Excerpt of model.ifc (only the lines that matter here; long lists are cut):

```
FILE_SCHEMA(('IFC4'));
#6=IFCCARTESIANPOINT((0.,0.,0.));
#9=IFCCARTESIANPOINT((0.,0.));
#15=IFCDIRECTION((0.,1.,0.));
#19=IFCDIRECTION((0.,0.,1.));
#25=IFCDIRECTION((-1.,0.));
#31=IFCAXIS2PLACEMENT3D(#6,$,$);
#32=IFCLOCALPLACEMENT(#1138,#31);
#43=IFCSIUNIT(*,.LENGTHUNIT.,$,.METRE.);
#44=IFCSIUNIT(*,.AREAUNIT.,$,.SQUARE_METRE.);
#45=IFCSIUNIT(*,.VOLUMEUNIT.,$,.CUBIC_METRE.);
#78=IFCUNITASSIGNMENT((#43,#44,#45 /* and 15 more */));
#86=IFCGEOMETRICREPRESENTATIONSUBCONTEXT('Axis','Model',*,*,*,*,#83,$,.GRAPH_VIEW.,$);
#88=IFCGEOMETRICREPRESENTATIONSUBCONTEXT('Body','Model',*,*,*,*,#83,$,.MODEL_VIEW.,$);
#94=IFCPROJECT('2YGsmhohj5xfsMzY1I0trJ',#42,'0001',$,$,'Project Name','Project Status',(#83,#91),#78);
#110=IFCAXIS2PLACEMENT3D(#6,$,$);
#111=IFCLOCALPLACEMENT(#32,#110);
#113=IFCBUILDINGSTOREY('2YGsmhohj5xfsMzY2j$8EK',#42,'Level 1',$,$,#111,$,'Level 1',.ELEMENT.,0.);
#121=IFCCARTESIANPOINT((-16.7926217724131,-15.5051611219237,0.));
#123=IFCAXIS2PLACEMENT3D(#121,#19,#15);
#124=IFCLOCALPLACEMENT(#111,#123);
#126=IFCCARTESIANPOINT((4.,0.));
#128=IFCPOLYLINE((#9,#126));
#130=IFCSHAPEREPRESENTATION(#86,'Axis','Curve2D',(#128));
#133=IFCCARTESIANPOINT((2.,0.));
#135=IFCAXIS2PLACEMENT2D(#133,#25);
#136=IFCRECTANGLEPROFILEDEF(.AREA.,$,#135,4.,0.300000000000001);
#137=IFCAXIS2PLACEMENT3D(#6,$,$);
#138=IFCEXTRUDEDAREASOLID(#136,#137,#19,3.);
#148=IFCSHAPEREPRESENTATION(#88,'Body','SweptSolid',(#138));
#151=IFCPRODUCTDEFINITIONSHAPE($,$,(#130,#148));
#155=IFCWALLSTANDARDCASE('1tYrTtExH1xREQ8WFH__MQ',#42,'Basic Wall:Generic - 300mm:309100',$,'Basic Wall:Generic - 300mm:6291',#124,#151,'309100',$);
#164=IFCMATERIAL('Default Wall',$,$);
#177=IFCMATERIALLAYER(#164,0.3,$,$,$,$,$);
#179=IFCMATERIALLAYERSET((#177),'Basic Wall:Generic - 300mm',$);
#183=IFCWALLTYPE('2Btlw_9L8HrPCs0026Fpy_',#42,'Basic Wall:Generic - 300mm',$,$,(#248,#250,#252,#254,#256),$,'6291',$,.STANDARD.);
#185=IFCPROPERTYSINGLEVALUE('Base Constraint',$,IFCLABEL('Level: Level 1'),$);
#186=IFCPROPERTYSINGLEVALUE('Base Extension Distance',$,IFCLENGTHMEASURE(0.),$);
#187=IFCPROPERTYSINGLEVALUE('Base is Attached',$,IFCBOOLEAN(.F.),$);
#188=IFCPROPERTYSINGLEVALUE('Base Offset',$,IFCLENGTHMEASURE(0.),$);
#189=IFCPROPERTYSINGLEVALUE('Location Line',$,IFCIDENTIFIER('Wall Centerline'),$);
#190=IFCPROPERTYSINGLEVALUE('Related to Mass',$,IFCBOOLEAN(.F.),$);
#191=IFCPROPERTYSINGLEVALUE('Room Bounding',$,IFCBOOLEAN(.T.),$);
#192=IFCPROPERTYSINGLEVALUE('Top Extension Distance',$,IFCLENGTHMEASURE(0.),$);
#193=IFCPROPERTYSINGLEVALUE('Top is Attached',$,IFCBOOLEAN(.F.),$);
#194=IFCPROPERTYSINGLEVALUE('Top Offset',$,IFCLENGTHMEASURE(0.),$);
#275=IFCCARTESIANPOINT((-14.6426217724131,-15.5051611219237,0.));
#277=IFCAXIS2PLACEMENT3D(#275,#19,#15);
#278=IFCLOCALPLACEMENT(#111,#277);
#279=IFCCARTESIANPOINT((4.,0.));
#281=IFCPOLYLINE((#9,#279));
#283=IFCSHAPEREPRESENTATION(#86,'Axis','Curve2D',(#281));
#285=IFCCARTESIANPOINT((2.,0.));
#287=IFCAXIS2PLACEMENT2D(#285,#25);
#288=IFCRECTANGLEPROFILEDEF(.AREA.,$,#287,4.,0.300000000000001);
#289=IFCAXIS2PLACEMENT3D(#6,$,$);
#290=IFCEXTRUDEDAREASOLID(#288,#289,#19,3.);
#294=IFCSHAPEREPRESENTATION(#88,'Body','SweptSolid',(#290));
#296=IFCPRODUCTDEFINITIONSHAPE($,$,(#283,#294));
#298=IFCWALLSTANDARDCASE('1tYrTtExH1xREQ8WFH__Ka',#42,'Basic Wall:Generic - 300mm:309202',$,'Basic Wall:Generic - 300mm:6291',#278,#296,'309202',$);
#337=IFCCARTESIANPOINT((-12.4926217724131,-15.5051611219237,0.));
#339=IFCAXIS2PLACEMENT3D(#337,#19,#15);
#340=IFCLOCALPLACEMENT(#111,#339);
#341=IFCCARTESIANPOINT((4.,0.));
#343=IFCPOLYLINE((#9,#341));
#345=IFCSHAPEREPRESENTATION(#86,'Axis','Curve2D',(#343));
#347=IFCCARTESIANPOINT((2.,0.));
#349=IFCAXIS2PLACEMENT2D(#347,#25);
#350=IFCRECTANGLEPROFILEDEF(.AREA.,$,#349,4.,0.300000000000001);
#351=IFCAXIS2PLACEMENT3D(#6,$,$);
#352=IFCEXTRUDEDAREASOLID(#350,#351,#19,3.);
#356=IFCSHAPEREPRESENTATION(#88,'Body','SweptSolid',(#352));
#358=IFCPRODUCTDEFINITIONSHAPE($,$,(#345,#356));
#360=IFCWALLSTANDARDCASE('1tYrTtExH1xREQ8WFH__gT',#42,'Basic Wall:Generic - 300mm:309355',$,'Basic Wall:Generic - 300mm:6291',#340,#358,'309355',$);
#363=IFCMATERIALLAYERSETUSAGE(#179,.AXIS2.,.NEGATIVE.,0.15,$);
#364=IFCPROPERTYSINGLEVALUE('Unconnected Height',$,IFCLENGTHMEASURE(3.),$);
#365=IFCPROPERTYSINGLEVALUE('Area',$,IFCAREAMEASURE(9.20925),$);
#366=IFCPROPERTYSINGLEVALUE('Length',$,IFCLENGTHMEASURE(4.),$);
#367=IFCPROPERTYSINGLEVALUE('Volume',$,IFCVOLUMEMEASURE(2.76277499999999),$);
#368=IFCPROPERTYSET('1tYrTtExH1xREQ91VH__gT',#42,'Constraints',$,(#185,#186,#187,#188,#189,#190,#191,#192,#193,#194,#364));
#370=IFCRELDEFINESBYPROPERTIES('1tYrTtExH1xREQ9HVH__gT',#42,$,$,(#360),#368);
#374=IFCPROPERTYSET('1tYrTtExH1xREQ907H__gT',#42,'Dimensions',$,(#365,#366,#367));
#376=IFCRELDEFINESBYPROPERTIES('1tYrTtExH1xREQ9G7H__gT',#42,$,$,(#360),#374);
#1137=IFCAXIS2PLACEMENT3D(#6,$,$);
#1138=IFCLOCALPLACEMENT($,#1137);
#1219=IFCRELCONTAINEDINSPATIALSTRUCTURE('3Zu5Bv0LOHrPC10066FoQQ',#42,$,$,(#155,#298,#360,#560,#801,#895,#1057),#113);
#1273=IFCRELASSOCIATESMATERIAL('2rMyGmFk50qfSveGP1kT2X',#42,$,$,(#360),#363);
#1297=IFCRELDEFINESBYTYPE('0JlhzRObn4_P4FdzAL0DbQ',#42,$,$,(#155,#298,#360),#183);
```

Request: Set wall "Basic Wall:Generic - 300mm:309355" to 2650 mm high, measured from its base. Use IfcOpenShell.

```python
import ifcopenshell
import ifcopenshell.api.pset
import ifcopenshell.geom
import ifcopenshell.util.element
import ifcopenshell.util.representation
import ifcopenshell.util.shape
import ifcopenshell.util.unit

model = ifcopenshell.open("model.ifc")
unit_scale = ifcopenshell.util.unit.calculate_unit_scale(model)
area_scale = ifcopenshell.util.unit.calculate_unit_scale(model, "AREAUNIT")
volume_scale = ifcopenshell.util.unit.calculate_unit_scale(model, "VOLUMEUNIT")
settings = ifcopenshell.geom.settings()


def volume(element):
    """Net volume in cubic metres, openings subtracted."""
    shape = ifcopenshell.geom.create_shape(settings, element)
    return ifcopenshell.util.shape.get_volume(shape.geometry)


wall = model.by_guid("1tYrTtExH1xREQ8WFH__gT")
before = volume(wall)

body = ifcopenshell.util.representation.get_representation(wall, "Model", "Body")
solid = body.Items[0]
old_height = solid.Depth
solid.Depth = 2.65 / unit_scale
after = volume(wall)
thickness = 0.3  # wall thickness in metres

# Update the stored height, areas and volumes.
pset = model.by_id(ifcopenshell.util.element.get_pset(wall, "Constraints", should_inherit=False)["id"])
ifcopenshell.api.pset.edit_pset(model, pset=pset, properties={
    "Unconnected Height": model.create_entity("IfcLengthMeasure", solid.Depth),
})
pset = model.by_id(ifcopenshell.util.element.get_pset(wall, "Dimensions", should_inherit=False)["id"])
ifcopenshell.api.pset.edit_pset(model, pset=pset, properties={
    "Area": model.create_entity("IfcAreaMeasure", after / thickness / area_scale),
    "Volume": model.create_entity("IfcVolumeMeasure", after / volume_scale),
})

print(f"height {old_height:g} -> {solid.Depth:g}, volume {before:.3f} -> {after:.3f} m3")

model.write("model_edited.ifc")
```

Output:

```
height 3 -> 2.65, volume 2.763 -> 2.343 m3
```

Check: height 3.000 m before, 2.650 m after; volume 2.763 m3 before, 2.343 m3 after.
